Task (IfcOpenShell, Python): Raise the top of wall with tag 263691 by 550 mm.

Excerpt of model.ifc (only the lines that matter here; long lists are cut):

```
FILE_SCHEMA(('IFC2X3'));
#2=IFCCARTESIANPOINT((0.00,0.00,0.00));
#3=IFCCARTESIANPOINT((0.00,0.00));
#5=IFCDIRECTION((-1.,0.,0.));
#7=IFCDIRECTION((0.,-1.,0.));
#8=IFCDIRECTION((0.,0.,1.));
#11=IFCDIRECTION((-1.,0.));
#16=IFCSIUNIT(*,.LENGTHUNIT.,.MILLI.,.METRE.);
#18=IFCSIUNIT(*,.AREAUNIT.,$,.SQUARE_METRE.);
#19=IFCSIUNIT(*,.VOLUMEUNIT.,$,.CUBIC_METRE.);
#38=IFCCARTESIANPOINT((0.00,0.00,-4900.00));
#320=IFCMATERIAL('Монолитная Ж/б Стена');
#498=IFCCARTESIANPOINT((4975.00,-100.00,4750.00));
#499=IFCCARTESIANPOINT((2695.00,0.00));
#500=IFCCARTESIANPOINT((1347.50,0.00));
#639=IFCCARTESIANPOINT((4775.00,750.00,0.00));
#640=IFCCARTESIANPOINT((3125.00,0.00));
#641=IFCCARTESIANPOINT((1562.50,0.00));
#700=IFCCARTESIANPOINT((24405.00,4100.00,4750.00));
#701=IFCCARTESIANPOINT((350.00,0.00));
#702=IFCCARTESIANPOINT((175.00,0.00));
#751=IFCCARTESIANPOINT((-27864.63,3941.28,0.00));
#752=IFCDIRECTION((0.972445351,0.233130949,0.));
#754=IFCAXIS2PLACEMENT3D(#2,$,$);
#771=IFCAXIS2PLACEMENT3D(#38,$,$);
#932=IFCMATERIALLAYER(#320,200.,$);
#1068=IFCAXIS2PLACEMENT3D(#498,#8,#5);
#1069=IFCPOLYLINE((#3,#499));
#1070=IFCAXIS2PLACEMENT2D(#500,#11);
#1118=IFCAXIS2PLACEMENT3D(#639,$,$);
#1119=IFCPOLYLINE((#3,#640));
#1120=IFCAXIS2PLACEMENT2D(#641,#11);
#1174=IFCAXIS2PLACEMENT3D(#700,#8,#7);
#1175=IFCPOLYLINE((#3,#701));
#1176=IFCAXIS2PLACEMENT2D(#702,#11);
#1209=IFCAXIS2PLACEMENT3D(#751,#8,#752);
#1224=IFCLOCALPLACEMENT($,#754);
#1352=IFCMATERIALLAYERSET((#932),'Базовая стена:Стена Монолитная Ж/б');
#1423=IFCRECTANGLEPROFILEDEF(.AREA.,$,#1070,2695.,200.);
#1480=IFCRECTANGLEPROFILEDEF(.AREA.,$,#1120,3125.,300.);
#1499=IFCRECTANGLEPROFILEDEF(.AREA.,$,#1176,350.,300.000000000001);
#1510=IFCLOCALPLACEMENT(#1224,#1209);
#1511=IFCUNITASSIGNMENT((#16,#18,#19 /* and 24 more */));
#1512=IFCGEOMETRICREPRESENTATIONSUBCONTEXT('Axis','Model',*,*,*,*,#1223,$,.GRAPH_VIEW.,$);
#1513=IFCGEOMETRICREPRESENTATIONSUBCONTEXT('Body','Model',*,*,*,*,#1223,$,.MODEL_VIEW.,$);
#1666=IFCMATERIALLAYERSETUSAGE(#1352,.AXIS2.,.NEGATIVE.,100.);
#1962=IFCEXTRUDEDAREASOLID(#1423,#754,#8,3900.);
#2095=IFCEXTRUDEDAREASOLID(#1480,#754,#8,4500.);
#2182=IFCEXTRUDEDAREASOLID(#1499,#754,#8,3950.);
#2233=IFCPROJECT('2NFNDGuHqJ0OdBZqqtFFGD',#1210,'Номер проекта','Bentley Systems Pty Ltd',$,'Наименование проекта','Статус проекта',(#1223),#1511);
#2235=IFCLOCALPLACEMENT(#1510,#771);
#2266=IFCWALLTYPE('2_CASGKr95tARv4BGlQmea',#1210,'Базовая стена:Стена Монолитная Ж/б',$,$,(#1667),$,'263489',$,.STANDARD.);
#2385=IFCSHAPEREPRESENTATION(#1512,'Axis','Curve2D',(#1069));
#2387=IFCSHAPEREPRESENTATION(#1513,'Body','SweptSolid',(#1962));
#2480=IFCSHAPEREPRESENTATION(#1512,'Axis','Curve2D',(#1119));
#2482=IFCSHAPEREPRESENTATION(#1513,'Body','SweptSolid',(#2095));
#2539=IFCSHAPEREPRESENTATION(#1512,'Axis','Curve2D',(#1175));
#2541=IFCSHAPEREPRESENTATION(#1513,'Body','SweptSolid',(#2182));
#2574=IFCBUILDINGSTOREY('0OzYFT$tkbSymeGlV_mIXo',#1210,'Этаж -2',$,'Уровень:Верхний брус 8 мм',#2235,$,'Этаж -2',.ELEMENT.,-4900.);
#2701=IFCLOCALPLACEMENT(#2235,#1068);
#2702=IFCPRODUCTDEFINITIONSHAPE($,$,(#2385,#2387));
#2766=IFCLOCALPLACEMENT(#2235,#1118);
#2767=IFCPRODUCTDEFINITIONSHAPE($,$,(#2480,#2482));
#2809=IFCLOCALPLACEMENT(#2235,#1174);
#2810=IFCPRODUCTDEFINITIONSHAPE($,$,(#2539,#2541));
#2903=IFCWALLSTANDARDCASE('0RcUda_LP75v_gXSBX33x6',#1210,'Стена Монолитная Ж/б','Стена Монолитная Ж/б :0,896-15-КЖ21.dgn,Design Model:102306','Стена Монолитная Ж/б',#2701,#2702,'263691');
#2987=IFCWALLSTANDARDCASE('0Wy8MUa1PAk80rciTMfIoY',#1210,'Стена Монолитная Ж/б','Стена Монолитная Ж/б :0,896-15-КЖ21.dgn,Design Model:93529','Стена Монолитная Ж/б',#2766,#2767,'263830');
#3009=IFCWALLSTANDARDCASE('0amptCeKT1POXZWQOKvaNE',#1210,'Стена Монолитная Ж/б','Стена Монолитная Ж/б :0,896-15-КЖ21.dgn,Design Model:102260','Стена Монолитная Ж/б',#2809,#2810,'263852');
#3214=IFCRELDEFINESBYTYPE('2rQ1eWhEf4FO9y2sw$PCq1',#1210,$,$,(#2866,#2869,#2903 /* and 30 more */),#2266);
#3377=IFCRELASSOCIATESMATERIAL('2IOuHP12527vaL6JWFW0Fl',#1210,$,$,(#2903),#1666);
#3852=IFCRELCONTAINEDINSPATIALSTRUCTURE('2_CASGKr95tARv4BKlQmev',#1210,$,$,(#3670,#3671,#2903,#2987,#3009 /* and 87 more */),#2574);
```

```python
import ifcopenshell
import ifcopenshell.geom
import ifcopenshell.util.representation
import ifcopenshell.util.shape
import ifcopenshell.util.unit

model = ifcopenshell.open("model.ifc")
unit_scale = ifcopenshell.util.unit.calculate_unit_scale(model)
settings = ifcopenshell.geom.settings()


def volume(element):
    """Net volume in cubic metres, openings subtracted."""
    shape = ifcopenshell.geom.create_shape(settings, element)
    return ifcopenshell.util.shape.get_volume(shape.geometry)


wall = model.by_id(2903)
before = volume(wall)

body = ifcopenshell.util.representation.get_representation(wall, "Model", "Body")
solid = body.Items[0]
old_height = solid.Depth
solid.Depth += 0.55 / unit_scale
after = volume(wall)

print(f"height {old_height:g} -> {solid.Depth:g}, volume {before:.3f} -> {after:.3f} m3")

model.write("model_updated.ifc")
```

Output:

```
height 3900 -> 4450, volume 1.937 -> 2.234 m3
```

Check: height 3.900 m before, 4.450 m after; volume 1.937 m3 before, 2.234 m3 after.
